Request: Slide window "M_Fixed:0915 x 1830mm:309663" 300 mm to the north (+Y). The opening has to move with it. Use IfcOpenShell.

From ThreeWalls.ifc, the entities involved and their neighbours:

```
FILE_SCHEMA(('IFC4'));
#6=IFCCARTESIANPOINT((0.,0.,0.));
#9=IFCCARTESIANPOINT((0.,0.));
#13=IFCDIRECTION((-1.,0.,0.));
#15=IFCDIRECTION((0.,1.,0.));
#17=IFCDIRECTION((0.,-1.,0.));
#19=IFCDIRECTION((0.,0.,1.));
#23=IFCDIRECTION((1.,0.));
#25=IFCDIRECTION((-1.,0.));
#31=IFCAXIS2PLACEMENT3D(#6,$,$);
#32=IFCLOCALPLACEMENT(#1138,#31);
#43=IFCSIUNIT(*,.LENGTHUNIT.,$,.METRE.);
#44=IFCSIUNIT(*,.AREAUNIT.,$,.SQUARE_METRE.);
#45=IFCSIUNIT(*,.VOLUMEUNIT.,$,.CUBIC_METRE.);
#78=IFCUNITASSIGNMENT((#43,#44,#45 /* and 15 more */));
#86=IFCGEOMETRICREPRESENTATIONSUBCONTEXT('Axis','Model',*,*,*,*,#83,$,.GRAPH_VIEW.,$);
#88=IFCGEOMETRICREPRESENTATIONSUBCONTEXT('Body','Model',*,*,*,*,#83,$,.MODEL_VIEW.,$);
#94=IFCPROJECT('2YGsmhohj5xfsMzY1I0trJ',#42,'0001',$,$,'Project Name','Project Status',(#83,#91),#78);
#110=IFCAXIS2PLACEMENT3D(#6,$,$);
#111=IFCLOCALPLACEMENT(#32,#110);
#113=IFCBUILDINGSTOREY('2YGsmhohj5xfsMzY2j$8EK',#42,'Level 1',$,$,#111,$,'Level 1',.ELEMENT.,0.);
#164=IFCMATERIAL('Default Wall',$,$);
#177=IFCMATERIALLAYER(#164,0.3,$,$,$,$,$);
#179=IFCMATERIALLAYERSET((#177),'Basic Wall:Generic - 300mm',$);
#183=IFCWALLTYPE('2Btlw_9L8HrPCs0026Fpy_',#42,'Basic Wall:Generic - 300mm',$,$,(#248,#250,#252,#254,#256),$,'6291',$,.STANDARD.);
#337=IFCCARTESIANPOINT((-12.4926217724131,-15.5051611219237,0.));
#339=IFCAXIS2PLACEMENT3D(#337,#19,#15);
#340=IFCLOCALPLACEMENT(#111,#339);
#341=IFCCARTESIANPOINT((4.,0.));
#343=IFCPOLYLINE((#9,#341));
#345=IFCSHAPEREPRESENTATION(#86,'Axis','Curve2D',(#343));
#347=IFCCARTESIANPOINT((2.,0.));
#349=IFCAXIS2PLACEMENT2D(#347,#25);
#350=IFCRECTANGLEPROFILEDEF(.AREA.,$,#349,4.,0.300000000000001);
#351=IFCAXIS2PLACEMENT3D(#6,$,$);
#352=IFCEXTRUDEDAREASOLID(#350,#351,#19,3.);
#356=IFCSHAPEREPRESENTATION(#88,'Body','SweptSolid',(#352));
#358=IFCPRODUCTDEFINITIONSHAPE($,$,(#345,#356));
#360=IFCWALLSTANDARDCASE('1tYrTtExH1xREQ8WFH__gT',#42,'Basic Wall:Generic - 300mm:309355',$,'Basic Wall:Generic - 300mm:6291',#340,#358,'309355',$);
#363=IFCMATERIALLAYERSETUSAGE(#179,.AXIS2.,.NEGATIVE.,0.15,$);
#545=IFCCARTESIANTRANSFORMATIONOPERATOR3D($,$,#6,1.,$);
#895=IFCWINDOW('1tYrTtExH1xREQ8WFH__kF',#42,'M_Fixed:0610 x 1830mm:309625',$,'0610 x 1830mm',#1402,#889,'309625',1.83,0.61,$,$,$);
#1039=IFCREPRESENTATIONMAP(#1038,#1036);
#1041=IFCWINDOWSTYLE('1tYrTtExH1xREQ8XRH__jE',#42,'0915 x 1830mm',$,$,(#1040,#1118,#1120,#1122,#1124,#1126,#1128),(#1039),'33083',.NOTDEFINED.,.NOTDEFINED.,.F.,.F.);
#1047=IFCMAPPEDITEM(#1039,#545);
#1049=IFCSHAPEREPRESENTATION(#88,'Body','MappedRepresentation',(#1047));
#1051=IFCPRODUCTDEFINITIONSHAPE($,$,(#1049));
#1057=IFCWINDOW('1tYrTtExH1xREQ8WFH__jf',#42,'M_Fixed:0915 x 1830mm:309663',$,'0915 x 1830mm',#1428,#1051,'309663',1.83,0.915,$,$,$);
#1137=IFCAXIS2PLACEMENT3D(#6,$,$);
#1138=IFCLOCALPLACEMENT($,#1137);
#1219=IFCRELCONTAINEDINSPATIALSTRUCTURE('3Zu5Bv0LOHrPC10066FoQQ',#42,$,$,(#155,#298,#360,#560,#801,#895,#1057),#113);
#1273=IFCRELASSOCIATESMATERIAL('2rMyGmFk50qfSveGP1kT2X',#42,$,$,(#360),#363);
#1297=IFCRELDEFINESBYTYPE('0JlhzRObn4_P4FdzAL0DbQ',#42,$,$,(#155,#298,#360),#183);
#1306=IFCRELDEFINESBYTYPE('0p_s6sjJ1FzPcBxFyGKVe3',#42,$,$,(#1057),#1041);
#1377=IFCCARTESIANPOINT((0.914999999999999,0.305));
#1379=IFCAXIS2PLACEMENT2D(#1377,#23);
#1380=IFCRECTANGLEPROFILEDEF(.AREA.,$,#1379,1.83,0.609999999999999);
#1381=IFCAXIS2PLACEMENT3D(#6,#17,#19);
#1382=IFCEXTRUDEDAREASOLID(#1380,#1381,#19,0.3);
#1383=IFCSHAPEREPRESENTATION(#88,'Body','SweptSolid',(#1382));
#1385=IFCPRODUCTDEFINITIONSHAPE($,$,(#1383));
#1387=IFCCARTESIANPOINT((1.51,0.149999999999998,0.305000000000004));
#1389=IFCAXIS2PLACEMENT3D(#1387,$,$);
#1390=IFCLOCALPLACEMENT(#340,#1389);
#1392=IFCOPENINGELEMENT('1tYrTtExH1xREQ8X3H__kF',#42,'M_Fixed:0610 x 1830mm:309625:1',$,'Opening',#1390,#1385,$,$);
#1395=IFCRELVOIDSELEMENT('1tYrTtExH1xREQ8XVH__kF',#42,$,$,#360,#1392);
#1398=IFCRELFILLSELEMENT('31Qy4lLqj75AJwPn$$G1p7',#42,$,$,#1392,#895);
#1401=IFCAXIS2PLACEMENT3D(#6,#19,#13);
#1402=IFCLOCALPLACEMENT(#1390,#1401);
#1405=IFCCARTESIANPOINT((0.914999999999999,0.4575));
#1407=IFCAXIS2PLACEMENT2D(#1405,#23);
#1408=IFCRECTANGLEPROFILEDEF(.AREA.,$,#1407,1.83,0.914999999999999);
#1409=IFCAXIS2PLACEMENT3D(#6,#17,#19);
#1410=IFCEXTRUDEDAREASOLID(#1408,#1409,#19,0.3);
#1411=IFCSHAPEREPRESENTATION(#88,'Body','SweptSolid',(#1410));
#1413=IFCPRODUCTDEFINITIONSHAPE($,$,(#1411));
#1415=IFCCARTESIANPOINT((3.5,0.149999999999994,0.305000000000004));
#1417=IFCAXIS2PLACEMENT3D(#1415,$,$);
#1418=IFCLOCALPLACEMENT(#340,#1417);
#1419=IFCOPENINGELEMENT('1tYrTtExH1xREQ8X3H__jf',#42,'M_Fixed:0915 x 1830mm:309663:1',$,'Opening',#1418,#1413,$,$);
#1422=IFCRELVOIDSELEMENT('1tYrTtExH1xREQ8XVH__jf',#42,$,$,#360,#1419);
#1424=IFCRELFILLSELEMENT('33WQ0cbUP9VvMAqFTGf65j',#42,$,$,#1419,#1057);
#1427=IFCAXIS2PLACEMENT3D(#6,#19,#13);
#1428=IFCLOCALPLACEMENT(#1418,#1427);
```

```python
import ifcopenshell
import ifcopenshell.api.geometry
import ifcopenshell.util.placement

model = ifcopenshell.open("ThreeWalls.ifc")

window = model.by_guid("1tYrTtExH1xREQ8WFH__jf")
opening = window.FillsVoids[0].RelatingOpeningElement
wall = opening.VoidsElements[0].RelatingBuildingElement

wall_matrix = ifcopenshell.util.placement.get_local_placement(wall.ObjectPlacement)
shift = wall_matrix[:3, 0] * 0.3
before = ifcopenshell.util.placement.get_local_placement(window.ObjectPlacement)[:3, 3].copy()

# The window is placed relative to its opening, so it follows when the opening moves.
matrix = ifcopenshell.util.placement.get_local_placement(opening.ObjectPlacement)
matrix[:3, 3] += shift
ifcopenshell.api.geometry.edit_object_placement(
    model, product=opening, matrix=matrix, is_si=False, should_transform_children=True
)

after = ifcopenshell.util.placement.get_local_placement(window.ObjectPlacement)[:3, 3]
print("window moved by", (after - before).round(3) + 0.0)

model.write("ThreeWalls_edited.ifc")
```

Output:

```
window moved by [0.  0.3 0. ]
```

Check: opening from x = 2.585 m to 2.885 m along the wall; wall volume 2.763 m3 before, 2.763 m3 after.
